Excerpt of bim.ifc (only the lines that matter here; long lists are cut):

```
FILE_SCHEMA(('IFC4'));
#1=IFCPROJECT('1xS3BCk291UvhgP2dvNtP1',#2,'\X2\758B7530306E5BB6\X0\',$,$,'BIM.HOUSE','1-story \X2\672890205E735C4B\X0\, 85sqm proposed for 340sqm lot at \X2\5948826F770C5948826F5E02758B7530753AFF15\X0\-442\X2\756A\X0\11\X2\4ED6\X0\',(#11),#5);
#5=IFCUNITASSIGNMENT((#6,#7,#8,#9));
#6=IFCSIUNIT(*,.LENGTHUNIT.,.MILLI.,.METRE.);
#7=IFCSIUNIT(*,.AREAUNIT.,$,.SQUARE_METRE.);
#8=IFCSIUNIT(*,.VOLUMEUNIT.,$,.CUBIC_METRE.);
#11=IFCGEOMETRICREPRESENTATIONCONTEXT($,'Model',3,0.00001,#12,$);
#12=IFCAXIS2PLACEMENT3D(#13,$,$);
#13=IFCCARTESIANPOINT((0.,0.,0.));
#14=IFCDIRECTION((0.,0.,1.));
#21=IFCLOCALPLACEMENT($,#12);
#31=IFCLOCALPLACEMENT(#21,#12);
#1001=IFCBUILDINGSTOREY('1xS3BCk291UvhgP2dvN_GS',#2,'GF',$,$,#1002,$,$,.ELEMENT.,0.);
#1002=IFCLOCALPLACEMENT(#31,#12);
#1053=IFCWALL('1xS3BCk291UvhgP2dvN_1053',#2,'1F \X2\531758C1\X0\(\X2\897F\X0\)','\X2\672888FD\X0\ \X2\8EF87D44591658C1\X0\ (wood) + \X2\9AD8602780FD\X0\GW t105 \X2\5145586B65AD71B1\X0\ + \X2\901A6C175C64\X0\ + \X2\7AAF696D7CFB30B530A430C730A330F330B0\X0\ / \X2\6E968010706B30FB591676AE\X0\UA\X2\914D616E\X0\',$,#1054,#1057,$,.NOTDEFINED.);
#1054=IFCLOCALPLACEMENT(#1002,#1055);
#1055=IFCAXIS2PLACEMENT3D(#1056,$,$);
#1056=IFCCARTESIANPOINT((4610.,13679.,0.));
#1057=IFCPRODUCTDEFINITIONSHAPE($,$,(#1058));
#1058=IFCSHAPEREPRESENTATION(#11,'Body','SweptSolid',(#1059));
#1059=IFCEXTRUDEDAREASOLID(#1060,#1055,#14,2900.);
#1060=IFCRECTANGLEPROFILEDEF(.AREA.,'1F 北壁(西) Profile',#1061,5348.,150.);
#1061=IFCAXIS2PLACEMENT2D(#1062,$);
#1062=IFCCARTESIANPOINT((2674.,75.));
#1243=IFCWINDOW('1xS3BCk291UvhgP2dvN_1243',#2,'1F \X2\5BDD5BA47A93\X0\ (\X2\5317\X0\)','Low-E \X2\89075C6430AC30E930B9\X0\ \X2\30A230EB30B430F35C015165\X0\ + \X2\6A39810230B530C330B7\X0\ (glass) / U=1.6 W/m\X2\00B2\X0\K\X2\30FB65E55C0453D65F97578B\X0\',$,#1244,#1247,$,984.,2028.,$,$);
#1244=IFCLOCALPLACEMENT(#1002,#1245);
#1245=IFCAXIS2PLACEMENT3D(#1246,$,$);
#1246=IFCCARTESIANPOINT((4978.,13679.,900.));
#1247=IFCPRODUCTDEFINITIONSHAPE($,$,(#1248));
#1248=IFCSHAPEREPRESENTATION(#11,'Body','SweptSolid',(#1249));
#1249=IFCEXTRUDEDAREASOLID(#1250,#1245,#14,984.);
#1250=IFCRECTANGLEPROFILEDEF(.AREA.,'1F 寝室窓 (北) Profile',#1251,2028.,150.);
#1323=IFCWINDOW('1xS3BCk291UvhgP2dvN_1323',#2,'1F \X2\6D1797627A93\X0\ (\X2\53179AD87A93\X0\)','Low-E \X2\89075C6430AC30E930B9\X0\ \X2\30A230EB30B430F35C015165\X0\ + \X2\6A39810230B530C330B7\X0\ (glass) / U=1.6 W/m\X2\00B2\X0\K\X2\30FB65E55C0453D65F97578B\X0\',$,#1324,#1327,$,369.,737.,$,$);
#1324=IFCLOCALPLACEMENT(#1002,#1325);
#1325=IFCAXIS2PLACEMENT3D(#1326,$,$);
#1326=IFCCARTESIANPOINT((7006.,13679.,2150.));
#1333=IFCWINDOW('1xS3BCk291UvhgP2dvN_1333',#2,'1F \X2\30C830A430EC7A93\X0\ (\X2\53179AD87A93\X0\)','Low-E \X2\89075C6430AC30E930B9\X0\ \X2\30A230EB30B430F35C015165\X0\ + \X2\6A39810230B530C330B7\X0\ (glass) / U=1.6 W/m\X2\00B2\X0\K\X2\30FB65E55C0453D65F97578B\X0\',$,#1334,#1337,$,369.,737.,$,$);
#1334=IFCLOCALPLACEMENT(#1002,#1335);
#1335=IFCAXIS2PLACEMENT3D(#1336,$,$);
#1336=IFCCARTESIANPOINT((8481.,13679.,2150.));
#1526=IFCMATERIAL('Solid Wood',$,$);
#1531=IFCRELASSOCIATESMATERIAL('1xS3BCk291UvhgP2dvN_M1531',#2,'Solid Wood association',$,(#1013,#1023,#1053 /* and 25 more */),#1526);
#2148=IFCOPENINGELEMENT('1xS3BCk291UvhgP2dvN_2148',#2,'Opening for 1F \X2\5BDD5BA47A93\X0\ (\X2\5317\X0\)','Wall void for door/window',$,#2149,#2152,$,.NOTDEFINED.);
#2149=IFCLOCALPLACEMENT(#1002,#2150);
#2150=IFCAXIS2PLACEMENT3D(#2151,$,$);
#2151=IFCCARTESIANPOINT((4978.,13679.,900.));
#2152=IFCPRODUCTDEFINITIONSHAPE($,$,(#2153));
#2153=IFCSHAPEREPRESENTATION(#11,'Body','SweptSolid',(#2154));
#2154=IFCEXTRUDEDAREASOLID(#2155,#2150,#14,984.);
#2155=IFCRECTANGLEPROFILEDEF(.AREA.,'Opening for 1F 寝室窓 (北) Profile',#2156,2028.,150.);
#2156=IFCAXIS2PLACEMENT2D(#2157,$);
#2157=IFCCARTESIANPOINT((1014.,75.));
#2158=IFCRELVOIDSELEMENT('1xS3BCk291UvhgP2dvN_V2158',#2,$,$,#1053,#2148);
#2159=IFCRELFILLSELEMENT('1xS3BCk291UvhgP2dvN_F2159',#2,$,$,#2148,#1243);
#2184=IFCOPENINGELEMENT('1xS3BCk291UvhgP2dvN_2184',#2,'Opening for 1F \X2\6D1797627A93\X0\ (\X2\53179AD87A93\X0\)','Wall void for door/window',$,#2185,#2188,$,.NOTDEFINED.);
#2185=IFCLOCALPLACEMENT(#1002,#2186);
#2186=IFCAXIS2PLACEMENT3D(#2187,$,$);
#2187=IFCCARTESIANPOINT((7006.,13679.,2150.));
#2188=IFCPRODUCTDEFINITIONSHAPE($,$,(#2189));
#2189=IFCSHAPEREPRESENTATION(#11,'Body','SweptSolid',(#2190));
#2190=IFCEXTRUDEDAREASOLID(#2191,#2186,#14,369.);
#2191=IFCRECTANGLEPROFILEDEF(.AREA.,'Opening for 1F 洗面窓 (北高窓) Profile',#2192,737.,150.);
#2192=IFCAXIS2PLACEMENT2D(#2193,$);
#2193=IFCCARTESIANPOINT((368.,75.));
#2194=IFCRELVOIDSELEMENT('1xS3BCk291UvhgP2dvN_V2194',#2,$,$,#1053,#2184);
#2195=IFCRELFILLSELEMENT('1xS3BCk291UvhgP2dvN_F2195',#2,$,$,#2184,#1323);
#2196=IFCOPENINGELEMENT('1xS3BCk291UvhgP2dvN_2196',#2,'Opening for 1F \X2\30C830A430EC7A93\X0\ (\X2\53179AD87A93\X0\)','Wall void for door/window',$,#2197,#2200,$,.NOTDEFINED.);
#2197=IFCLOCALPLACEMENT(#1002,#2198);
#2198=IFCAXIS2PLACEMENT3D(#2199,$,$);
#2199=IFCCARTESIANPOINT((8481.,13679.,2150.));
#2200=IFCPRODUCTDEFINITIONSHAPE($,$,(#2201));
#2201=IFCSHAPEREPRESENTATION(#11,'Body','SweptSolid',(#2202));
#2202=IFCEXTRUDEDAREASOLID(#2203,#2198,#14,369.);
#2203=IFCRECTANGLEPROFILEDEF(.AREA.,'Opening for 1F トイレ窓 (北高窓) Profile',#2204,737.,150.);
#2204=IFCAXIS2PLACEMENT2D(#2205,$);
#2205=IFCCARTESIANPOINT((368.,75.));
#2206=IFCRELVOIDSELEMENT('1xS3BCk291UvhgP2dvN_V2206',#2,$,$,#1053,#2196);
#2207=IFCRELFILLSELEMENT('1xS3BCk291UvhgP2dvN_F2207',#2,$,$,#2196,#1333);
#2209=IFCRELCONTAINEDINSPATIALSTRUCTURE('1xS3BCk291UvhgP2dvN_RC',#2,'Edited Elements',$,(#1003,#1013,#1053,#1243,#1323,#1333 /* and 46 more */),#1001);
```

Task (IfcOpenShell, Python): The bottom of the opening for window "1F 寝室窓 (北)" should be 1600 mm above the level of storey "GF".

```python
import numpy as np
import ifcopenshell
import ifcopenshell.api.geometry
import ifcopenshell.geom
import ifcopenshell.util.element
import ifcopenshell.util.placement
import ifcopenshell.util.shape
import ifcopenshell.util.unit

model = ifcopenshell.open("bim.ifc")
unit_scale = ifcopenshell.util.unit.calculate_unit_scale(model)

window = model.by_id(1243)
opening = window.FillsVoids[0].RelatingOpeningElement
storey = ifcopenshell.util.element.get_container(window, ifc_class="IfcBuildingStorey")
level = ifcopenshell.util.placement.get_local_placement(storey.ObjectPlacement)[2, 3]

# The opening's origin need not be at the sill, so measure its lowest point.
shape = ifcopenshell.geom.create_shape(ifcopenshell.geom.settings(), opening)
bottom = ifcopenshell.util.shape.get_shape_bottom_elevation(shape, shape.geometry) / unit_scale
dz = level + 1.6 / unit_scale - bottom

shift = np.array([0.0, 0.0, dz])
# The window is not placed relative to its opening, so move both.
for product in (opening, window):
    matrix = ifcopenshell.util.placement.get_local_placement(product.ObjectPlacement)
    matrix[:3, 3] += shift
    ifcopenshell.api.geometry.edit_object_placement(model, product=product, matrix=matrix, is_si=False)

print(f"moved by {dz * unit_scale:+.3f} m")

model.write("bim-out.ifc")
```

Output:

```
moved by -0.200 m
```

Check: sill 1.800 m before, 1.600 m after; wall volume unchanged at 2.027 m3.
